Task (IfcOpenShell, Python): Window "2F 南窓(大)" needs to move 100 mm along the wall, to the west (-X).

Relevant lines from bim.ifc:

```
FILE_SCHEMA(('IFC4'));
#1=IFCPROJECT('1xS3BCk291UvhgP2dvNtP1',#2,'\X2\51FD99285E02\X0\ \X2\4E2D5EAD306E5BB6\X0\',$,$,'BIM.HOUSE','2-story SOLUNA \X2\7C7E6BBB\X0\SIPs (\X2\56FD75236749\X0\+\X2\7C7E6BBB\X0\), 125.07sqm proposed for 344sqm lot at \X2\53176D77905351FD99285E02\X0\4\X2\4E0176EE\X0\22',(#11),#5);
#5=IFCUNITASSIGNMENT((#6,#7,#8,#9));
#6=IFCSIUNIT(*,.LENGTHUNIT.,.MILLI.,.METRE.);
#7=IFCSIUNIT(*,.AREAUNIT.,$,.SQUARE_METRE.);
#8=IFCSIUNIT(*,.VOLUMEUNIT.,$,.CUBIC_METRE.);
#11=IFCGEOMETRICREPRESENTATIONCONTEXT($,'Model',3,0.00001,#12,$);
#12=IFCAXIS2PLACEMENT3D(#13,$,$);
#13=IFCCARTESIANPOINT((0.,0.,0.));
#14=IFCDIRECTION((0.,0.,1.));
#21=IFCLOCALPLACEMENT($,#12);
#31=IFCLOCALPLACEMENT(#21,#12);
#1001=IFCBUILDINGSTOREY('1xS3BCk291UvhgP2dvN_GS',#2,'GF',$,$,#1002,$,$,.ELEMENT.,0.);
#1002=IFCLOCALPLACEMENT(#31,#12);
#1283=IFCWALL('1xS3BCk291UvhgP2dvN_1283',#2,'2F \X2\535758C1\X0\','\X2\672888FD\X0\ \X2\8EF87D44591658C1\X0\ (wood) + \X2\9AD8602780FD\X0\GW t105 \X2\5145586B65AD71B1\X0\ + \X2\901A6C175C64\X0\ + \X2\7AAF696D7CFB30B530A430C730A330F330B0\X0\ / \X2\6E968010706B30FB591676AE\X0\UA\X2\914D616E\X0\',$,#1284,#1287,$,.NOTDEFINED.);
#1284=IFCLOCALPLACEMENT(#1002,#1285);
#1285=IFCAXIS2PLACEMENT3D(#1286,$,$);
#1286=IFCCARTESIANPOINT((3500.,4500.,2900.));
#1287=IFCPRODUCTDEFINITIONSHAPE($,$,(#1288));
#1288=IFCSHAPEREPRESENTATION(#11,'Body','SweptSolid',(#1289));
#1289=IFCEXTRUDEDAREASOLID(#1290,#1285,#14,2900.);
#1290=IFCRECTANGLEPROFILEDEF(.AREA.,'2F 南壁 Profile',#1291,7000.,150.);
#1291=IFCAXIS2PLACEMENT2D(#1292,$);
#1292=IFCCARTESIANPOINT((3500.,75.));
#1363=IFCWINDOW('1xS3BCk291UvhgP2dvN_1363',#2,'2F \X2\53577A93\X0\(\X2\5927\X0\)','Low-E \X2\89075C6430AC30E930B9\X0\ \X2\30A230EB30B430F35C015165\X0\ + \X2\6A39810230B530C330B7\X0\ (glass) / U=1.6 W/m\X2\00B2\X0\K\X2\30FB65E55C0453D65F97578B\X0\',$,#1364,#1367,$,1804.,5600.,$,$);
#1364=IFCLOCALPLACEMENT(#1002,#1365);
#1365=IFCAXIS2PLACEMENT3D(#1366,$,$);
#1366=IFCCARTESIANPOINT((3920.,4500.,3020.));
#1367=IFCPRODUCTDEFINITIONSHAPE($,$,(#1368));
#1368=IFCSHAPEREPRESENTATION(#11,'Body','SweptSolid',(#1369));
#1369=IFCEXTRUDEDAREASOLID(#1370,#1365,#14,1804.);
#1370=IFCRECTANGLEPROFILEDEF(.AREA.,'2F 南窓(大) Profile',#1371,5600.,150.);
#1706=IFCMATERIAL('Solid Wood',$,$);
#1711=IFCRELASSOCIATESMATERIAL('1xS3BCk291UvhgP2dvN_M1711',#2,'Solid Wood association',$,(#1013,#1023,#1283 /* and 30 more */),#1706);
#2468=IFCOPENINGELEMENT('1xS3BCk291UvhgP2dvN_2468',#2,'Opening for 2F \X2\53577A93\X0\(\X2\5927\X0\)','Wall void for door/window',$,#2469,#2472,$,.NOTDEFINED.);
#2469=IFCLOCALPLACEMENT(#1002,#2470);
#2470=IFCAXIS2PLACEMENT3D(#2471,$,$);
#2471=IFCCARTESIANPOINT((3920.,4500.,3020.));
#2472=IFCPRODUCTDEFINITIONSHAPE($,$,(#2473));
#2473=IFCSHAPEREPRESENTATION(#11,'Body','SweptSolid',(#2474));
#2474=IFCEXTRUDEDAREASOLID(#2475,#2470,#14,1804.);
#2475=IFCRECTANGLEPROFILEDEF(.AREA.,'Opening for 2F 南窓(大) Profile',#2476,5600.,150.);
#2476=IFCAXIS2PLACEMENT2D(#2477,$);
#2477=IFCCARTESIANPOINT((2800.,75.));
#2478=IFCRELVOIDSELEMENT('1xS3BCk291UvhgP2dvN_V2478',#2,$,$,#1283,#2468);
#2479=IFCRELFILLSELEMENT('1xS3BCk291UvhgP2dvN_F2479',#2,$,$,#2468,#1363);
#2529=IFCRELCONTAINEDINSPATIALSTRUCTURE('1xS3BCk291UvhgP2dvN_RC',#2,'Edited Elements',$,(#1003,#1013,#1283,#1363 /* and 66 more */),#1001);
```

```python
import ifcopenshell
import ifcopenshell.api.geometry
import ifcopenshell.util.placement

model = ifcopenshell.open("bim.ifc")

window = model.by_id(1363)
opening = window.FillsVoids[0].RelatingOpeningElement
wall = opening.VoidsElements[0].RelatingBuildingElement

wall_matrix = ifcopenshell.util.placement.get_local_placement(wall.ObjectPlacement)
shift = wall_matrix[:3, 0] * -100.0
before = ifcopenshell.util.placement.get_local_placement(window.ObjectPlacement)[:3, 3].copy()

# The window is not placed relative to its opening, so move both.
for product in (opening, window):
    matrix = ifcopenshell.util.placement.get_local_placement(product.ObjectPlacement)
    matrix[:3, 3] += shift
    ifcopenshell.api.geometry.edit_object_placement(model, product=product, matrix=matrix, is_si=False)

after = ifcopenshell.util.placement.get_local_placement(window.ObjectPlacement)[:3, 3]
print("window moved by", (after - before).round(3) + 0.0)

model.write("bim_rev.ifc")
```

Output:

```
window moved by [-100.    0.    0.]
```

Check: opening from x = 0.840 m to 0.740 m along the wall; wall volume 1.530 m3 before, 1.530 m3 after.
